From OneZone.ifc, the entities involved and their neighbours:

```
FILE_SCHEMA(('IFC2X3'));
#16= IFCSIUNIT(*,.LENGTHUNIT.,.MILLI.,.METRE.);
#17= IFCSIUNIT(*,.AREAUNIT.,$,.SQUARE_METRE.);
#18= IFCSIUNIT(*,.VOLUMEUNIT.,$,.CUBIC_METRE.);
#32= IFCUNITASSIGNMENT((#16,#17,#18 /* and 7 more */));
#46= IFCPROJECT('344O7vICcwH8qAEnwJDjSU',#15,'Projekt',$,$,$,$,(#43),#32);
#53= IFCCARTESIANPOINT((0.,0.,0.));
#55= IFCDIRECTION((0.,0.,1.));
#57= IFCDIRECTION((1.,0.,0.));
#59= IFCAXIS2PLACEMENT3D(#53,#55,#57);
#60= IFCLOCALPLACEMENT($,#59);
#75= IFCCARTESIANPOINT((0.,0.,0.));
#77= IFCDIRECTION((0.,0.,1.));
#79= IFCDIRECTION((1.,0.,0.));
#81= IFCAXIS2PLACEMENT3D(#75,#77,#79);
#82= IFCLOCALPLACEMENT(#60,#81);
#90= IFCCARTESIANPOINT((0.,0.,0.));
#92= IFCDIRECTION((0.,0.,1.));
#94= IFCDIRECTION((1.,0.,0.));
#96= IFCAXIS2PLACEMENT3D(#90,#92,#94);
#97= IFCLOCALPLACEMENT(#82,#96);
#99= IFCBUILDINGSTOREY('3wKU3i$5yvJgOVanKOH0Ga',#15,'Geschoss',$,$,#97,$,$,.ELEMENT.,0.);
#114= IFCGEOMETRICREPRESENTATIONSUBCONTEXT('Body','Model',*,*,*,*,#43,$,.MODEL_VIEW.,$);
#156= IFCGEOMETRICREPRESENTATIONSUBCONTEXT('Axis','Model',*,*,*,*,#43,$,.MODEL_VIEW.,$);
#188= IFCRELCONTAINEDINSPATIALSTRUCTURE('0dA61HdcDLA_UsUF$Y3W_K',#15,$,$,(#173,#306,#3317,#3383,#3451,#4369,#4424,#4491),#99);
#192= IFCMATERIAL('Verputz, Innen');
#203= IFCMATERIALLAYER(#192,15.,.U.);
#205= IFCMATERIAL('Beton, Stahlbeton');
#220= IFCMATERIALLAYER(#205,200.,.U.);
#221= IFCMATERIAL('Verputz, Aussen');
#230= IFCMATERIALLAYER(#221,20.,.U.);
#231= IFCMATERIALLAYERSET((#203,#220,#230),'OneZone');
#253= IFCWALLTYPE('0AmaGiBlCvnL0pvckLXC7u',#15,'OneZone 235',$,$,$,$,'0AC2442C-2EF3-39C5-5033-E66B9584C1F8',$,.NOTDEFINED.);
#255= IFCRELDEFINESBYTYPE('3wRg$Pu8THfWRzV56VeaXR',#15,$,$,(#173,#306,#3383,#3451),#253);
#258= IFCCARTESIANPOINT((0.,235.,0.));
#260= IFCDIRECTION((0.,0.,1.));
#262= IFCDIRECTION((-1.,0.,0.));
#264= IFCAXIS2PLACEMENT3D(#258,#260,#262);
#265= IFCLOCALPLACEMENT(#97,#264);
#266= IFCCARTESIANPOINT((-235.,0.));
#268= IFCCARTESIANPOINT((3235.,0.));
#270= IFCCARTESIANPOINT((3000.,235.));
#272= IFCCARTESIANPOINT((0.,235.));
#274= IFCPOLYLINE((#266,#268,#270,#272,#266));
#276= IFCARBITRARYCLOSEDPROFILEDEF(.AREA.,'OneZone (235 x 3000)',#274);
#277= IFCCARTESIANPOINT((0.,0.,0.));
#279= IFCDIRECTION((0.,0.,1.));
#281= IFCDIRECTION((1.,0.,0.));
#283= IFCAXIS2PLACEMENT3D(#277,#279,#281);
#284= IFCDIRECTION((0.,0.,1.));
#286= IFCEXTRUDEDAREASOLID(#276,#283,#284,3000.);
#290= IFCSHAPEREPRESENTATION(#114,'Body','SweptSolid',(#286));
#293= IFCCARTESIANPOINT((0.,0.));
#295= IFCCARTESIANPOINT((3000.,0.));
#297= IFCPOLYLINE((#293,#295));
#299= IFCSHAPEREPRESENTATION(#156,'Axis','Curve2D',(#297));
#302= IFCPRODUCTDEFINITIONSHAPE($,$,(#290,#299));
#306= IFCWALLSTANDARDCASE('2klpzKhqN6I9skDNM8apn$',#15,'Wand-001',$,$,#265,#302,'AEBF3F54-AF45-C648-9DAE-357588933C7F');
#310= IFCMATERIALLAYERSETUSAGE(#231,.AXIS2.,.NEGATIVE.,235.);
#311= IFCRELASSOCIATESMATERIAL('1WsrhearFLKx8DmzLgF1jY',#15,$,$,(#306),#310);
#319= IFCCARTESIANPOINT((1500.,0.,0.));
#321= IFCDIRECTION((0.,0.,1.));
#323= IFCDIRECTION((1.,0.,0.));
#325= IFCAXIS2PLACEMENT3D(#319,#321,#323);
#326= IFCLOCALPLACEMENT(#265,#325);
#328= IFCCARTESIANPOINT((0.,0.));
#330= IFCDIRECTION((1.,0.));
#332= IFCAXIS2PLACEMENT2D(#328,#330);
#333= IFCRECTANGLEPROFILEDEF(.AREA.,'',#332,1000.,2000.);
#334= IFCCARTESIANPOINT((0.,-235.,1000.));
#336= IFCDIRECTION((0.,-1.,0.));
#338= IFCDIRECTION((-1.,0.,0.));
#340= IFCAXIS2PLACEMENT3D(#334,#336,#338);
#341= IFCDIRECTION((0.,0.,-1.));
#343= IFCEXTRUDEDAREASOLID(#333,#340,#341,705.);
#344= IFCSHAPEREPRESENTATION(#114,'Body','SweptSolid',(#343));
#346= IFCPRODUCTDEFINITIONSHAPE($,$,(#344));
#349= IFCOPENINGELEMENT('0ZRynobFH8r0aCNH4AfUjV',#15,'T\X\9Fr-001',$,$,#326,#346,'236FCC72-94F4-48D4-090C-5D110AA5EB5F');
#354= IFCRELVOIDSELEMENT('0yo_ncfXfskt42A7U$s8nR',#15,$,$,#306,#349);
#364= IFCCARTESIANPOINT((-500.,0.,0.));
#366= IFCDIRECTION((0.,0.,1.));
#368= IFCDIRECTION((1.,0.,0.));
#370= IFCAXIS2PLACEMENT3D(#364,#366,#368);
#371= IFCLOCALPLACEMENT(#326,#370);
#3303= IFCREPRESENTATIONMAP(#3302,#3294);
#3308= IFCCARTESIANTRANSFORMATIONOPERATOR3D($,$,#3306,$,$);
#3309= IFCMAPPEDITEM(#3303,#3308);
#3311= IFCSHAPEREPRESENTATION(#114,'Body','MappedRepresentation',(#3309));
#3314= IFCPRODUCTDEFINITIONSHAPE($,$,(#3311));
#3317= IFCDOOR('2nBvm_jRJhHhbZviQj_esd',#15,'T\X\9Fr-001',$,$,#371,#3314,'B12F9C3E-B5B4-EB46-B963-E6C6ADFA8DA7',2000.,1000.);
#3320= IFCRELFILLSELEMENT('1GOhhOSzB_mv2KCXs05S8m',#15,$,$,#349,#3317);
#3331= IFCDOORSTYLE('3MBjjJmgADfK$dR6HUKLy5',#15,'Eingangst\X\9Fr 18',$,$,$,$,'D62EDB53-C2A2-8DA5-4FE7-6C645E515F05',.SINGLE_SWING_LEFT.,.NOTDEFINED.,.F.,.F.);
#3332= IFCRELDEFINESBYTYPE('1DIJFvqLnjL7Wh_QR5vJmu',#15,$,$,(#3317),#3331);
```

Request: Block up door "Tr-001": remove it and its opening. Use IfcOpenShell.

```python
import ifcopenshell
import ifcopenshell.api.feature
import ifcopenshell.api.root
import ifcopenshell.geom
import ifcopenshell.util.shape

model = ifcopenshell.open("OneZone.ifc")
settings = ifcopenshell.geom.settings()


def volume(element):
    """Net volume in cubic metres, openings subtracted."""
    shape = ifcopenshell.geom.create_shape(settings, element)
    return ifcopenshell.util.shape.get_volume(shape.geometry)


door = model.by_guid("2nBvm_jRJhHhbZviQj_esd")
opening = door.FillsVoids[0].RelatingOpeningElement
wall = opening.VoidsElements[0].RelatingBuildingElement
before = volume(wall)

ifcopenshell.api.root.remove_product(model, product=door)
ifcopenshell.api.feature.remove_feature(model, feature=opening)

after = volume(wall)

print(f"wall volume {before:.3f} -> {after:.3f} m3")

model.write("OneZone_updated.ifc")
```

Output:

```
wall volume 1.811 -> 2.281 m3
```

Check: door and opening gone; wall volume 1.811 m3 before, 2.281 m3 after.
